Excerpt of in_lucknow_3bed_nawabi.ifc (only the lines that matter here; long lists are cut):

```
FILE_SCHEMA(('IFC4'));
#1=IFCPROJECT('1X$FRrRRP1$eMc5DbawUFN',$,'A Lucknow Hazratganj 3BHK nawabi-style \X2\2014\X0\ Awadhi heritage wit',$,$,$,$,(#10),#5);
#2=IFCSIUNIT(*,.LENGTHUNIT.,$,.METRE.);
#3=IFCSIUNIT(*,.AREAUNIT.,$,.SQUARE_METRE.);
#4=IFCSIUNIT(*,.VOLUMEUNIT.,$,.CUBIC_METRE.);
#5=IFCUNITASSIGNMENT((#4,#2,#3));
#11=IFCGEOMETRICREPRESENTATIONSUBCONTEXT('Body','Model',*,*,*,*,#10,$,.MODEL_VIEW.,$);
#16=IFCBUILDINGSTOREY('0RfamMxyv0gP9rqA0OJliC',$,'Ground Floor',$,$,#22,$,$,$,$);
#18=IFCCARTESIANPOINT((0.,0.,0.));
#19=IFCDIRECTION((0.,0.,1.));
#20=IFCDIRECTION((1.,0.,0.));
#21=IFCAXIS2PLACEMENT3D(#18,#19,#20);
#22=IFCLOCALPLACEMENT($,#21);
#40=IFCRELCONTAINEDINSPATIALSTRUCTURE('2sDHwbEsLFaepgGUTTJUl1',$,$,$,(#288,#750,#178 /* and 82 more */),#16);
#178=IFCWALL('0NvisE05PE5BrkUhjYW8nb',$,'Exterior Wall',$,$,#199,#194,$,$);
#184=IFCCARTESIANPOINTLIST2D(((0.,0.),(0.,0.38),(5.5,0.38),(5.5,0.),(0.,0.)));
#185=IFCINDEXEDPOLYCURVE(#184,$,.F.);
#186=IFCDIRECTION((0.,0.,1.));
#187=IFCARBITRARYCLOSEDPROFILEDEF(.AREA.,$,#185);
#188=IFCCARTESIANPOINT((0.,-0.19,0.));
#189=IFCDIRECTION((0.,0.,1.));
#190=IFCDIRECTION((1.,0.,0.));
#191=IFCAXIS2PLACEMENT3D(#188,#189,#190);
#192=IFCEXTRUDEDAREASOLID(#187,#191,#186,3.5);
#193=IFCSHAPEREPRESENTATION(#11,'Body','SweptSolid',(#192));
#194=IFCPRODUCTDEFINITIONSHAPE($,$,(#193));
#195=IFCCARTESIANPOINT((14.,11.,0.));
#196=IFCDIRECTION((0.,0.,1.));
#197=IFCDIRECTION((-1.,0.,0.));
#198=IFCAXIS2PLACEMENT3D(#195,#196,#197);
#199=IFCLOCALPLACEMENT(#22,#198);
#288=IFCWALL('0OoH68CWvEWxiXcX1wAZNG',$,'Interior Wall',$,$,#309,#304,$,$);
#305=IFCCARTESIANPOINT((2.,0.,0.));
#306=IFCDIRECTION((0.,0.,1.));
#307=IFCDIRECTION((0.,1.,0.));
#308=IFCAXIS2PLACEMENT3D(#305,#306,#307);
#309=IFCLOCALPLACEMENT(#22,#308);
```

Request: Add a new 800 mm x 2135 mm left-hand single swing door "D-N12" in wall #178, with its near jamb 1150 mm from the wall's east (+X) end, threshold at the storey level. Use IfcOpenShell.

```python
import numpy as np
import ifcopenshell
import ifcopenshell.api.feature
import ifcopenshell.api.geometry
import ifcopenshell.api.root
import ifcopenshell.api.spatial
import ifcopenshell.geom
import ifcopenshell.util.element
import ifcopenshell.util.placement
import ifcopenshell.util.representation
import ifcopenshell.util.shape
import ifcopenshell.util.unit

model = ifcopenshell.open("in_lucknow_3bed_nawabi.ifc")
unit_scale = ifcopenshell.util.unit.calculate_unit_scale(model)
settings = ifcopenshell.geom.settings()


def volume(element):
    """Net volume in cubic metres, openings subtracted."""
    shape = ifcopenshell.geom.create_shape(settings, element)
    return ifcopenshell.util.shape.get_volume(shape.geometry)


wall = model.by_guid("0NvisE05PE5BrkUhjYW8nb")
storey = ifcopenshell.util.element.get_container(wall, ifc_class="IfcBuildingStorey")
context = ifcopenshell.util.representation.get_context(model, "Model", "Body", "MODEL_VIEW")
before = volume(wall)

width, height, from_end, sill = 0.8, 2.135, 1.15, 0.0  # metres

# The wall runs along its own X axis, and the end named is its -X end.
wall_shape = ifcopenshell.geom.create_shape(settings, wall)
x, y, z = ifcopenshell.util.shape.get_vertices(wall_shape.geometry).T
start = x.min() + from_end
face, thickness = float(y.min()), float(y.max() - y.min())
wall_matrix = ifcopenshell.util.placement.get_local_placement(wall.ObjectPlacement)
level = ifcopenshell.util.placement.get_local_placement(storey.ObjectPlacement)[2, 3]


def in_wall(x, y):
    """Placement at x, y metres in the wall's axes, at sill height."""
    matrix = wall_matrix.copy()
    matrix[:, 3] = wall_matrix @ np.array([x / unit_scale, y / unit_scale, 0.0, 1.0])
    matrix[2, 3] = level + sill / unit_scale
    return matrix


# Opening: a box that overshoots both wall faces by 50 mm.
opening = ifcopenshell.api.root.create_entity(model, ifc_class="IfcOpeningElement", predefined_type="OPENING")
box = ifcopenshell.api.geometry.add_wall_representation(
    model, context=context, length=width, height=height, thickness=thickness + 0.1
)
ifcopenshell.api.geometry.assign_representation(model, product=opening, representation=box)
ifcopenshell.api.geometry.edit_object_placement(model, product=opening, matrix=in_wall(start, face - 0.05), is_si=False)
ifcopenshell.api.feature.add_feature(model, feature=opening, element=wall)

door = ifcopenshell.api.root.create_entity(model, ifc_class="IfcDoor", name="D-N12", predefined_type="DOOR")
door.OverallWidth, door.OverallHeight = width / unit_scale, height / unit_scale
door.OperationType = "SINGLE_SWING_LEFT"
body = ifcopenshell.api.geometry.add_door_representation(
    model,
    context=context,
    overall_width=door.OverallWidth,
    overall_height=door.OverallHeight,
    operation_type="SINGLE_SWING_LEFT",
    lining_properties={"LiningDepth": thickness / unit_scale, "ThresholdDepth": thickness / unit_scale},
)
ifcopenshell.api.geometry.assign_representation(model, product=door, representation=body)
ifcopenshell.api.spatial.assign_container(model, products=[door], relating_structure=storey)
ifcopenshell.api.feature.add_filling(model, opening=opening, element=door)

# The lining spans the wall, so the door starts at the wall face.
ifcopenshell.api.geometry.edit_object_placement(model, product=door, matrix=in_wall(start, face), is_si=False)

after = volume(wall)

print(f"wall volume {before:.3f} -> {after:.3f} m3")

model.write("in_lucknow_3bed_nawabi_edited.ifc")
```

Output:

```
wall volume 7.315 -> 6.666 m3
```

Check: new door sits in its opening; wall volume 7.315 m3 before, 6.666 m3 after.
